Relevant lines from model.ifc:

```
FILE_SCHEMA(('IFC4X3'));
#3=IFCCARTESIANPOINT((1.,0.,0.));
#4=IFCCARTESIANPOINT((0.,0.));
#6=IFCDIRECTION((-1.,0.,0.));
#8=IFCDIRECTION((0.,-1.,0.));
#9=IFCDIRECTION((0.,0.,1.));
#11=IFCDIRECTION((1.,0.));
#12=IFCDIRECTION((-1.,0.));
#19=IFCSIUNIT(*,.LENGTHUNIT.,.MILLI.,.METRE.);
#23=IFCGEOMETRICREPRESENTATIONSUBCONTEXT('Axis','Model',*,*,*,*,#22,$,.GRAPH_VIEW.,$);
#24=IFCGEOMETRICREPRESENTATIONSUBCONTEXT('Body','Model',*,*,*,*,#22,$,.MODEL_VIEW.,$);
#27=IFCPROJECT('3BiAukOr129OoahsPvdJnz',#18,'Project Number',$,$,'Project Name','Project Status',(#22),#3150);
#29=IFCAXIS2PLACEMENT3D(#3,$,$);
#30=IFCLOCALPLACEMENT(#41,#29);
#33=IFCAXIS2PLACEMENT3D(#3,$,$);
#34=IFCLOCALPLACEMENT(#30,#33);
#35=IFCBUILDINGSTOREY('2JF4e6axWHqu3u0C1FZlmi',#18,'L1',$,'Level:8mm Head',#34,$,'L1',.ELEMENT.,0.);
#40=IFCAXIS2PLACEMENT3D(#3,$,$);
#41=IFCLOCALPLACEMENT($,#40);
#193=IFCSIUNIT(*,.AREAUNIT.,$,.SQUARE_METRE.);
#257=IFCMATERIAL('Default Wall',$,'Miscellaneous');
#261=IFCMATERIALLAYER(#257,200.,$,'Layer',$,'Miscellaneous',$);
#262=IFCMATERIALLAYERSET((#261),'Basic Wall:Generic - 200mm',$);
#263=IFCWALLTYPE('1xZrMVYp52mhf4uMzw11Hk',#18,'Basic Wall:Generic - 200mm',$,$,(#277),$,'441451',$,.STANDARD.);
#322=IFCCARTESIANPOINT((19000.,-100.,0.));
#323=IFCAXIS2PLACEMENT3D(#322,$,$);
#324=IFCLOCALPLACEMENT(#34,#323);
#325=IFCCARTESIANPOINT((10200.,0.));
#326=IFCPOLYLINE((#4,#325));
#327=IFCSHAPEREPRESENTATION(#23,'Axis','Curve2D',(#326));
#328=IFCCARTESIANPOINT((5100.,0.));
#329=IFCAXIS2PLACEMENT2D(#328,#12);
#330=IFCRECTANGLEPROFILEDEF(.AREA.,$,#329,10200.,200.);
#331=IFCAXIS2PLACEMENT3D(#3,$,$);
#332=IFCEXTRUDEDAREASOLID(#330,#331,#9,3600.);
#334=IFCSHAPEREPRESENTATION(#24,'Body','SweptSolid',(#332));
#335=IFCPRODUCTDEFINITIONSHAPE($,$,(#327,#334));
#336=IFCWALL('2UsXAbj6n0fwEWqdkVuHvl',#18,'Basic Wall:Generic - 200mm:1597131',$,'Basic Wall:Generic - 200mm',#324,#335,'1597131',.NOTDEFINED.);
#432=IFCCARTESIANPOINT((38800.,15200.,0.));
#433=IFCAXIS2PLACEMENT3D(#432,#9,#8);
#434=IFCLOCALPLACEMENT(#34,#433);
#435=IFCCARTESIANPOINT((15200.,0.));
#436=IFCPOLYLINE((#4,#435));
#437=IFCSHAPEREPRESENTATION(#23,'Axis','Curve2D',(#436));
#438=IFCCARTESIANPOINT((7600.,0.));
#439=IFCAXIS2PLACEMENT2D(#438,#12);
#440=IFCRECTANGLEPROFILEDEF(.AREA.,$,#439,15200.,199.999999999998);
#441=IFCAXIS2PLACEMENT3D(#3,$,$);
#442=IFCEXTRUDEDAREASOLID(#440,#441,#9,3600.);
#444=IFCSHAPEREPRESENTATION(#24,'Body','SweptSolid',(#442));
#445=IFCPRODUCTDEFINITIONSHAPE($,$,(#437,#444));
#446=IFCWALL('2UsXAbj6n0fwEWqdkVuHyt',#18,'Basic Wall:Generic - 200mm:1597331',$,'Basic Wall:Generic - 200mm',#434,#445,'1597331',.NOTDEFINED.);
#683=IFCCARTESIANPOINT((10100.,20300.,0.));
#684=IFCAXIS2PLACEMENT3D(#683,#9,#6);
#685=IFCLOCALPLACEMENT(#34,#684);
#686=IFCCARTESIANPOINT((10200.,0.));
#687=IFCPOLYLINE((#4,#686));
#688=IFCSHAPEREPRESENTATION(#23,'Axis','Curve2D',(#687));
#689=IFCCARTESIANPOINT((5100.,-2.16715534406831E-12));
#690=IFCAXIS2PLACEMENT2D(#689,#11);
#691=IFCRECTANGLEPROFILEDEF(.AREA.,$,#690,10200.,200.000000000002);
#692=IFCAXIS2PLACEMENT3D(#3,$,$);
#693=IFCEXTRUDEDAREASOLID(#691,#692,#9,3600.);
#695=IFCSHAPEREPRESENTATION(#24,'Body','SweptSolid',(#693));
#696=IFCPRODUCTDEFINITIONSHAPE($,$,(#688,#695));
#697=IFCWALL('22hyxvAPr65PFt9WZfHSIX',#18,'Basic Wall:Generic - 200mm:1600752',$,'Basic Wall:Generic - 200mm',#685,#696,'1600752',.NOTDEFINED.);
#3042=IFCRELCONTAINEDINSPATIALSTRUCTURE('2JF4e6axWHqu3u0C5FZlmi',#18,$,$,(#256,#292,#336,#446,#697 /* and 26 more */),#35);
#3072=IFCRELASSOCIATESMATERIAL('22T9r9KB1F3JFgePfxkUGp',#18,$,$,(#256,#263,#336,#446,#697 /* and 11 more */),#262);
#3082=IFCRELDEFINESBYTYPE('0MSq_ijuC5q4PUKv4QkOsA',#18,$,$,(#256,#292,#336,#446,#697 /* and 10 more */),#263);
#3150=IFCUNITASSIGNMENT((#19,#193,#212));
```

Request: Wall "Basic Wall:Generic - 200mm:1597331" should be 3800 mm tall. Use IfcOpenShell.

```python
import ifcopenshell
import ifcopenshell.geom
import ifcopenshell.util.representation
import ifcopenshell.util.shape

model = ifcopenshell.open("model.ifc")
settings = ifcopenshell.geom.settings()


def volume(element):
    """Net volume in cubic metres, openings subtracted."""
    shape = ifcopenshell.geom.create_shape(settings, element)
    return ifcopenshell.util.shape.get_volume(shape.geometry)


wall = model.by_guid("2UsXAbj6n0fwEWqdkVuHyt")
before = volume(wall)

body = ifcopenshell.util.representation.get_representation(wall, "Model", "Body")
solid = body.Items[0]
old_height = solid.Depth
solid.Depth = 3800.0
after = volume(wall)

print(f"height {old_height:g} -> {solid.Depth:g}, volume {before:.3f} -> {after:.3f} m3")

model.write("model_edited.ifc")
```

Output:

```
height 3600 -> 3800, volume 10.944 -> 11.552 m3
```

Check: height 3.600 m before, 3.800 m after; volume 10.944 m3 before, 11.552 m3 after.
